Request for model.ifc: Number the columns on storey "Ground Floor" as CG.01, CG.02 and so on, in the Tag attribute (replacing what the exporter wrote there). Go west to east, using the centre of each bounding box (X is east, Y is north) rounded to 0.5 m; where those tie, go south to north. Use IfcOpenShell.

First a look at what the model holds.

```python
import ifcopenshell
import ifcopenshell.util.element
import ifcopenshell.util.placement

model = ifcopenshell.open("model.ifc")
print(model.schema)
storey = next(s for s in model.by_type("IfcBuildingStorey") if s.Name == "Ground Floor")
columns = [e for e in ifcopenshell.util.element.get_decomposition(storey) if e.is_a("IfcColumn")]
for e in sorted(columns, key=lambda e: e.id()):
    origin = ifcopenshell.util.placement.get_local_placement(e.ObjectPlacement)[:3, 3]
    print(e.id(), e.Tag, e.Name, origin.round(2) + 0.0, sep=" | ")
```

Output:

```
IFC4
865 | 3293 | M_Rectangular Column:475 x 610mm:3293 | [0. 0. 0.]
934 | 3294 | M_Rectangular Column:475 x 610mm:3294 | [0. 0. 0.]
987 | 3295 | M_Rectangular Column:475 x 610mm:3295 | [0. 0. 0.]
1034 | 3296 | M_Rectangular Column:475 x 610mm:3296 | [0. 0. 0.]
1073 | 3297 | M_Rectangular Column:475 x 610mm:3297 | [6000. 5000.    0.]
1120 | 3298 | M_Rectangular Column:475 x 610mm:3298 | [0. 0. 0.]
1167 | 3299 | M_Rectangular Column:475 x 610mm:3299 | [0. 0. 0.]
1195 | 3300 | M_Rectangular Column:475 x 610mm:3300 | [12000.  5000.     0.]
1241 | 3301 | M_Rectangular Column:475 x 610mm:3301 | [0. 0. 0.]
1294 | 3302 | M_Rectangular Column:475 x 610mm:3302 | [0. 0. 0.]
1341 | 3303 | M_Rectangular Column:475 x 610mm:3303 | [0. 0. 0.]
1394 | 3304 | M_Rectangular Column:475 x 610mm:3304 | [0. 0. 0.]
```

```python
import ifcopenshell
import ifcopenshell.geom
import ifcopenshell.util.element
import ifcopenshell.util.shape

model = ifcopenshell.open("model.ifc")
settings = ifcopenshell.geom.settings()
settings.set("use-world-coords", True)


def centre(element):
    shape = ifcopenshell.geom.create_shape(settings, element)
    return ifcopenshell.util.shape.get_bbox_centroid(shape.geometry)


storey = next(s for s in model.by_type("IfcBuildingStorey") if s.Name == "Ground Floor")
columns = [e for e in ifcopenshell.util.element.get_decomposition(storey) if e.is_a("IfcColumn")]

# Insertion points can sit at a corner or the storey origin, so sort by the geometry (in metres).
centres = {e: centre(e) for e in columns}
columns.sort(key=lambda e: (round(centres[e][0] / 0.5), centres[e][1]))

for i, e in enumerate(columns, start=1):
    number = f"CG.{i:02d}"
    e.Tag = number
    print(e.id(), number)

model.write("model_edited.ifc")
```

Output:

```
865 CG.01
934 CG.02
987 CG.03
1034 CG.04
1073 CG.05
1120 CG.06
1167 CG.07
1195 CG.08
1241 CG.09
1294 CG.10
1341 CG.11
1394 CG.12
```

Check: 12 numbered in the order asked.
